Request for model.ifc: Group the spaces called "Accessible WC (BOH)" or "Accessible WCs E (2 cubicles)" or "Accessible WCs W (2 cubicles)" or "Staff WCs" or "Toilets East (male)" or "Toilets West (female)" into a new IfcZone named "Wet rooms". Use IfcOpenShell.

First a look at what the model holds.

```python
import ifcopenshell

model = ifcopenshell.open("model.ifc")
print(model.schema)
seen = {}
for space in model.by_type("IfcSpace"):
    seen[space.LongName] = seen.get(space.LongName, 0) + 1
for name, count in sorted(seen.items(), key=str):
    print(count, "x", name)
print("zones:", [z.Name for z in model.by_type("IfcZone")][:20])
```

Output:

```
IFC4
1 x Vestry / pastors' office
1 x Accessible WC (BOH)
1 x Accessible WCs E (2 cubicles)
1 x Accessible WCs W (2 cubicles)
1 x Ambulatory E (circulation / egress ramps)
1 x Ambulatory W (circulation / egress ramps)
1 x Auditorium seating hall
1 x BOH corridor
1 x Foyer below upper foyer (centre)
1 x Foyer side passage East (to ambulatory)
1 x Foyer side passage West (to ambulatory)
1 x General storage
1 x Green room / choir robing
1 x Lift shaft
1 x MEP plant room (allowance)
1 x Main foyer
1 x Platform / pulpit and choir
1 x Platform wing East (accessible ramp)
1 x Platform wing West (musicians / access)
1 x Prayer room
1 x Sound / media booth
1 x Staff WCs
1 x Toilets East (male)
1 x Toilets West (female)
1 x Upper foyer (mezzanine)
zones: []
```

```python
import ifcopenshell
import ifcopenshell.api.group
import ifcopenshell.api.root

model = ifcopenshell.open("model.ifc")

names = {"Accessible WC (BOH)", "Accessible WCs E (2 cubicles)", "Accessible WCs W (2 cubicles)", "Staff WCs", "Toilets East (male)", "Toilets West (female)"}
spaces = [s for s in model.by_type("IfcSpace") if s.LongName in names]

zone = ifcopenshell.api.root.create_entity(model, ifc_class="IfcZone", name="Wet rooms")
ifcopenshell.api.group.assign_group(model, products=spaces, group=zone)
print(len(spaces), "spaces in", zone.Name)

model.write("model_rev.ifc")
```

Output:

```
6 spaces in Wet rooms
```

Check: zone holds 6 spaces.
